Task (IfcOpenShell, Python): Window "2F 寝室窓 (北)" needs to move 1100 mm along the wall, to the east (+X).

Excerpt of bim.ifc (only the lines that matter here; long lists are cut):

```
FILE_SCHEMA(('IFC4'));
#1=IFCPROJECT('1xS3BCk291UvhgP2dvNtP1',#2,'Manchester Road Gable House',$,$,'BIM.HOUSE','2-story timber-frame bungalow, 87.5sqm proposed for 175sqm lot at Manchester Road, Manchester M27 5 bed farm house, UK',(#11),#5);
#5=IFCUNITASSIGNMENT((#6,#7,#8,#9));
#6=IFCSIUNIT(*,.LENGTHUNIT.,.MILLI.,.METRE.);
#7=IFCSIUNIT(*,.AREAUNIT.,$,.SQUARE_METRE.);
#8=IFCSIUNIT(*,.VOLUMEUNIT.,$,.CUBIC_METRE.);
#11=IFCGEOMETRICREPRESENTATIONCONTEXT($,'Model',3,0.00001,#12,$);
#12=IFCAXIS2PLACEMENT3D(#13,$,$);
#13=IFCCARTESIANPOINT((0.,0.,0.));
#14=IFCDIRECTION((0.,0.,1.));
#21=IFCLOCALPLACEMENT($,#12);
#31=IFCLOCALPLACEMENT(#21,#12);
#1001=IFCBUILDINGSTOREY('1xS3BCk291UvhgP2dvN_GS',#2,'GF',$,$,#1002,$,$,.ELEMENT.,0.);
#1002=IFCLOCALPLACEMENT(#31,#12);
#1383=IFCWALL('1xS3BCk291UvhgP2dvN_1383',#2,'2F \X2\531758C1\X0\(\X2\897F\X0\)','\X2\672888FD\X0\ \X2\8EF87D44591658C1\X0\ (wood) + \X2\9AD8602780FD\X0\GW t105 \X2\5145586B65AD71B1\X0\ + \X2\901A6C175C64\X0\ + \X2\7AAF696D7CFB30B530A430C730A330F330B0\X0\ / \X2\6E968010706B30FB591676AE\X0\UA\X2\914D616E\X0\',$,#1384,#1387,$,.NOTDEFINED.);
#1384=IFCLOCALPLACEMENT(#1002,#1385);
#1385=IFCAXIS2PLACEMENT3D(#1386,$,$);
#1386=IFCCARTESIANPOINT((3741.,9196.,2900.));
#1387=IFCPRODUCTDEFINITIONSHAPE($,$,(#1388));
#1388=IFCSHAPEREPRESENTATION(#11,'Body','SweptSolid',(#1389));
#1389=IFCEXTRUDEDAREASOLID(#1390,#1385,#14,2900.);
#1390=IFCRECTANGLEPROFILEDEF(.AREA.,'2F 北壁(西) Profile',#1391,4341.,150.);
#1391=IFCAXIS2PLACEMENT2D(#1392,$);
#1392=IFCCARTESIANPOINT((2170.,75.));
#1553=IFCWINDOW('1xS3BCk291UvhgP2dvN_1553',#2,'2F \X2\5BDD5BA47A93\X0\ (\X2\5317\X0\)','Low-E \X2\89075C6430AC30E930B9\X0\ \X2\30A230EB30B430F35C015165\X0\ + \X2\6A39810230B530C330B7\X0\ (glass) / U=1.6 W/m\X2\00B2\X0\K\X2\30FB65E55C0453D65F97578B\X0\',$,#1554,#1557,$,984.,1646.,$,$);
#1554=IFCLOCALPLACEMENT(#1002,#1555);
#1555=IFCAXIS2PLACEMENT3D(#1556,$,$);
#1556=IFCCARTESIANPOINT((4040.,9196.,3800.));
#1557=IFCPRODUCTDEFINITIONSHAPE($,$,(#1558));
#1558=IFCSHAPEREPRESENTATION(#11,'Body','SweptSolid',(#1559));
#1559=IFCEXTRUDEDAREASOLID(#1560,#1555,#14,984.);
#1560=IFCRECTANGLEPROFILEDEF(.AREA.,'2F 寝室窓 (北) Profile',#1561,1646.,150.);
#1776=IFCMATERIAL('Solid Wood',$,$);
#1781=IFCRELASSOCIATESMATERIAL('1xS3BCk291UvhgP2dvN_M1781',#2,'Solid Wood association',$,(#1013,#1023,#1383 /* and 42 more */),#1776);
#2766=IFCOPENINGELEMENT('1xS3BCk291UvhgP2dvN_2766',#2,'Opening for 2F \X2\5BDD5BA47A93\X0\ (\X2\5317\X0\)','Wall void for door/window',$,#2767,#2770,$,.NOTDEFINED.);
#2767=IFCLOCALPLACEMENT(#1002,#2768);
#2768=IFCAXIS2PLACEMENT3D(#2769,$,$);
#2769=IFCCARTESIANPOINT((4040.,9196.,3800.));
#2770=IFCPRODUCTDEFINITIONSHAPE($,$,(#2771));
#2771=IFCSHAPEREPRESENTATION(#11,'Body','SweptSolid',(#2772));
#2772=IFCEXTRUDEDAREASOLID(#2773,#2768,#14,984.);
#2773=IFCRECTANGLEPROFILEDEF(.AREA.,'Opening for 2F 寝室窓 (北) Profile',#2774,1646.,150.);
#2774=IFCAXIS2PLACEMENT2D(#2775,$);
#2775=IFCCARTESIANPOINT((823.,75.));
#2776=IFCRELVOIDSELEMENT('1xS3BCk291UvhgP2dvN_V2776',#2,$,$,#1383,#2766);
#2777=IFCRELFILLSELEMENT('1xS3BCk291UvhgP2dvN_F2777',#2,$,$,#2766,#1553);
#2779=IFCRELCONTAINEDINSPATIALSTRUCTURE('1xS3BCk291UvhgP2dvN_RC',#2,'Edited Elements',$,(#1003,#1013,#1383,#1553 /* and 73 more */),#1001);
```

```python
import ifcopenshell
import ifcopenshell.api.geometry
import ifcopenshell.util.placement

model = ifcopenshell.open("bim.ifc")

window = model.by_guid("1xS3BCk291UvhgP2dvN_1553")
opening = window.FillsVoids[0].RelatingOpeningElement
wall = opening.VoidsElements[0].RelatingBuildingElement

wall_matrix = ifcopenshell.util.placement.get_local_placement(wall.ObjectPlacement)
shift = wall_matrix[:3, 0] * 1100.0
before = ifcopenshell.util.placement.get_local_placement(window.ObjectPlacement)[:3, 3].copy()

# The window is not placed relative to its opening, so move both.
for product in (opening, window):
    matrix = ifcopenshell.util.placement.get_local_placement(product.ObjectPlacement)
    matrix[:3, 3] += shift
    ifcopenshell.api.geometry.edit_object_placement(model, product=product, matrix=matrix, is_si=False)

after = ifcopenshell.util.placement.get_local_placement(window.ObjectPlacement)[:3, 3]
print("window moved by", (after - before).round(3) + 0.0)

model.write("bim_edited.ifc")
```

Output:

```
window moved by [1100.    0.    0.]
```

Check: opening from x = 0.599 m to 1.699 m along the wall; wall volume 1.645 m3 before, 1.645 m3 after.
